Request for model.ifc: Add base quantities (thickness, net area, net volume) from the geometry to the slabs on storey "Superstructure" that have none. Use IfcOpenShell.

First a look at what the model holds.

```python
import ifcopenshell
import ifcopenshell.util.element
import ifcopenshell.util.unit

model = ifcopenshell.open("model.ifc")
print(model.schema)
for unit_type in ("LENGTHUNIT", "AREAUNIT", "VOLUMEUNIT"):
    print(unit_type, ifcopenshell.util.unit.calculate_unit_scale(model, unit_type))
storey = next(s for s in model.by_type("IfcBuildingStorey") if s.Name == "Superstructure")
slabs = [e for e in ifcopenshell.util.element.get_decomposition(storey) if e.is_a("IfcSlab")]
for e in sorted(slabs, key=lambda e: e.id()):
    print(e.id(), e.is_a(), e.Name, list(ifcopenshell.util.element.get_psets(e, qtos_only=True)), sep=" | ")
```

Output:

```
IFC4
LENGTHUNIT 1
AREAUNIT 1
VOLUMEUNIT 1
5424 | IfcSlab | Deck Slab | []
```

```python
import ifcopenshell
import ifcopenshell.api.pset
import ifcopenshell.geom
import ifcopenshell.util.element
import ifcopenshell.util.shape
import ifcopenshell.util.unit

model = ifcopenshell.open("model.ifc")
unit_scale = ifcopenshell.util.unit.calculate_unit_scale(model)
area_scale = ifcopenshell.util.unit.calculate_unit_scale(model, "AREAUNIT")
volume_scale = ifcopenshell.util.unit.calculate_unit_scale(model, "VOLUMEUNIT")
settings = ifcopenshell.geom.settings()

storey = next(s for s in model.by_type("IfcBuildingStorey") if s.Name == "Superstructure")
slabs = [e for e in ifcopenshell.util.element.get_decomposition(storey) if e.is_a("IfcSlab")]

for e in sorted(slabs, key=lambda e: e.id()):
    if ifcopenshell.util.element.get_psets(e, qtos_only=True, should_inherit=False):
        continue
    # Geometry comes back in metres, in the element's own axes.
    shape = ifcopenshell.geom.create_shape(settings, e)
    values = {
        "Width": ifcopenshell.util.shape.get_z(shape.geometry) / unit_scale,
        "NetArea": ifcopenshell.util.shape.get_footprint_area(shape.geometry) / area_scale,
        "NetVolume": ifcopenshell.util.shape.get_volume(shape.geometry) / volume_scale,
    }
    qto = ifcopenshell.api.pset.add_qto(model, product=e, name="Qto_SlabBaseQuantities")
    ifcopenshell.api.pset.edit_qto(model, qto=qto, properties=values)
    print(e.id(), {k: round(v, 3) for k, v in values.items()})

model.write("model_updated.ifc")
```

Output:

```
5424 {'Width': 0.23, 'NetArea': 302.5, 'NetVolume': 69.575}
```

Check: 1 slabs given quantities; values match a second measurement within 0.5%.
